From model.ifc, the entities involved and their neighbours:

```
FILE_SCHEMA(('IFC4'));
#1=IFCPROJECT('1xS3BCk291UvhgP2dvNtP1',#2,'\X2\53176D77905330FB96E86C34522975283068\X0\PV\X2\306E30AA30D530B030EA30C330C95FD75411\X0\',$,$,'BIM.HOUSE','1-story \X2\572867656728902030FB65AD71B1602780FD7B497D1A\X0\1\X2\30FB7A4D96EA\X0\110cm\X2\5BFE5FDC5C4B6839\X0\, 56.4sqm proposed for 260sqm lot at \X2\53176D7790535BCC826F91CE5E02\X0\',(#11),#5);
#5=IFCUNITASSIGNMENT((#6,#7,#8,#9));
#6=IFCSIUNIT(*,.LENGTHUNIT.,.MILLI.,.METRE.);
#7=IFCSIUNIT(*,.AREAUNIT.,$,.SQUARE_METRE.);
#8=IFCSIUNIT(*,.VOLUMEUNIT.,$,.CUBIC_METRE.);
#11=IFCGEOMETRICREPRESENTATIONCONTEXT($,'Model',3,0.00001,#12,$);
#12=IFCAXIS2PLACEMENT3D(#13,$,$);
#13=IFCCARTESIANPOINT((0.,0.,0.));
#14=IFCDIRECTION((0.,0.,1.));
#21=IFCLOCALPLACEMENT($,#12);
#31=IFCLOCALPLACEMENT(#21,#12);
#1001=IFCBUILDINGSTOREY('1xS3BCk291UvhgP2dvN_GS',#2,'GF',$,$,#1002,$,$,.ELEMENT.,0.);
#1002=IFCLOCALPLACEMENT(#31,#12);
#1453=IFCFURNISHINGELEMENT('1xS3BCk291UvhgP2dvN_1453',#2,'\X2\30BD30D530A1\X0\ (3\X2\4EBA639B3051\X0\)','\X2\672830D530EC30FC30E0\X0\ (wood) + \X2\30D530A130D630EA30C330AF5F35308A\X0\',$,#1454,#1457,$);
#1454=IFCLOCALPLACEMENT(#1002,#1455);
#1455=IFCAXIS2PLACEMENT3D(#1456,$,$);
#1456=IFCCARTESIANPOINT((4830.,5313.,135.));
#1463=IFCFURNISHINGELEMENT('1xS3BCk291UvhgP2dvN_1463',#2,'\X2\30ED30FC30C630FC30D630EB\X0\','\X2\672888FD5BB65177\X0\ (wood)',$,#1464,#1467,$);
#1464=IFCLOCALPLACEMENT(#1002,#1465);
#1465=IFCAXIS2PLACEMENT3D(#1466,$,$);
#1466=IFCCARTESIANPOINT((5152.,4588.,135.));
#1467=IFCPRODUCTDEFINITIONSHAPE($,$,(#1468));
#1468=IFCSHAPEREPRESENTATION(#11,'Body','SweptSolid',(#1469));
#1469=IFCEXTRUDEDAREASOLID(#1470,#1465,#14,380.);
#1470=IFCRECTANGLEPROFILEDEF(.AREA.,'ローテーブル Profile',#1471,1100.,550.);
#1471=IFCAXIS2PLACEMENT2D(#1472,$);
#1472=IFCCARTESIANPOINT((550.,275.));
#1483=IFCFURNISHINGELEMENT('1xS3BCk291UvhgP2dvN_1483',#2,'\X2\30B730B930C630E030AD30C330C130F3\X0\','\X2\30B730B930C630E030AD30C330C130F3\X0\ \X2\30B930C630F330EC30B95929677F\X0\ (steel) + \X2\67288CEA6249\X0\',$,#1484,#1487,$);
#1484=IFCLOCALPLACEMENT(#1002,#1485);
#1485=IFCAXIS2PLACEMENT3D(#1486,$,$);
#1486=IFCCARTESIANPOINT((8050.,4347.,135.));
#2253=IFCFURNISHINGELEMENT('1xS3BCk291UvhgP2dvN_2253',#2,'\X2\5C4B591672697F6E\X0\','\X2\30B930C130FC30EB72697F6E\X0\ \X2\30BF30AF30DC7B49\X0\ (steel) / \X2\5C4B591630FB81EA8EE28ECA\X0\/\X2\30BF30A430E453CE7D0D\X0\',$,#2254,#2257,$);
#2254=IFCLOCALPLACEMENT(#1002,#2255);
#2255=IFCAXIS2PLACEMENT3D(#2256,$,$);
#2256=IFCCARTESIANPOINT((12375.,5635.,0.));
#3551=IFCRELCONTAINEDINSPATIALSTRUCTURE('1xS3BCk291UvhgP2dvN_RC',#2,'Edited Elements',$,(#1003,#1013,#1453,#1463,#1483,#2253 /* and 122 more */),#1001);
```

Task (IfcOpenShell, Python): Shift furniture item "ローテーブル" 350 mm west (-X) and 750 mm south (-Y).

```python
import ifcopenshell
import ifcopenshell.api.geometry
import ifcopenshell.util.placement
import ifcopenshell.util.unit

model = ifcopenshell.open("model.ifc")
unit_scale = ifcopenshell.util.unit.calculate_unit_scale(model)

item = model.by_guid("1xS3BCk291UvhgP2dvN_1463")
matrix = ifcopenshell.util.placement.get_local_placement(item.ObjectPlacement)
matrix[0, 3] -= 0.35 / unit_scale
matrix[1, 3] -= 0.75 / unit_scale
ifcopenshell.api.geometry.edit_object_placement(model, product=item, matrix=matrix, is_si=False)

print(ifcopenshell.util.placement.get_local_placement(item.ObjectPlacement).round(3) + 0.0)

model.write("model_updated.ifc")
```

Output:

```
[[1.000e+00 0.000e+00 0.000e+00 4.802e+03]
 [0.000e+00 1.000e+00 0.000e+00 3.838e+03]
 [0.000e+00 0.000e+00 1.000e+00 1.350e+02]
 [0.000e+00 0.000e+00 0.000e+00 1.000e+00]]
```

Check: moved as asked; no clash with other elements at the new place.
